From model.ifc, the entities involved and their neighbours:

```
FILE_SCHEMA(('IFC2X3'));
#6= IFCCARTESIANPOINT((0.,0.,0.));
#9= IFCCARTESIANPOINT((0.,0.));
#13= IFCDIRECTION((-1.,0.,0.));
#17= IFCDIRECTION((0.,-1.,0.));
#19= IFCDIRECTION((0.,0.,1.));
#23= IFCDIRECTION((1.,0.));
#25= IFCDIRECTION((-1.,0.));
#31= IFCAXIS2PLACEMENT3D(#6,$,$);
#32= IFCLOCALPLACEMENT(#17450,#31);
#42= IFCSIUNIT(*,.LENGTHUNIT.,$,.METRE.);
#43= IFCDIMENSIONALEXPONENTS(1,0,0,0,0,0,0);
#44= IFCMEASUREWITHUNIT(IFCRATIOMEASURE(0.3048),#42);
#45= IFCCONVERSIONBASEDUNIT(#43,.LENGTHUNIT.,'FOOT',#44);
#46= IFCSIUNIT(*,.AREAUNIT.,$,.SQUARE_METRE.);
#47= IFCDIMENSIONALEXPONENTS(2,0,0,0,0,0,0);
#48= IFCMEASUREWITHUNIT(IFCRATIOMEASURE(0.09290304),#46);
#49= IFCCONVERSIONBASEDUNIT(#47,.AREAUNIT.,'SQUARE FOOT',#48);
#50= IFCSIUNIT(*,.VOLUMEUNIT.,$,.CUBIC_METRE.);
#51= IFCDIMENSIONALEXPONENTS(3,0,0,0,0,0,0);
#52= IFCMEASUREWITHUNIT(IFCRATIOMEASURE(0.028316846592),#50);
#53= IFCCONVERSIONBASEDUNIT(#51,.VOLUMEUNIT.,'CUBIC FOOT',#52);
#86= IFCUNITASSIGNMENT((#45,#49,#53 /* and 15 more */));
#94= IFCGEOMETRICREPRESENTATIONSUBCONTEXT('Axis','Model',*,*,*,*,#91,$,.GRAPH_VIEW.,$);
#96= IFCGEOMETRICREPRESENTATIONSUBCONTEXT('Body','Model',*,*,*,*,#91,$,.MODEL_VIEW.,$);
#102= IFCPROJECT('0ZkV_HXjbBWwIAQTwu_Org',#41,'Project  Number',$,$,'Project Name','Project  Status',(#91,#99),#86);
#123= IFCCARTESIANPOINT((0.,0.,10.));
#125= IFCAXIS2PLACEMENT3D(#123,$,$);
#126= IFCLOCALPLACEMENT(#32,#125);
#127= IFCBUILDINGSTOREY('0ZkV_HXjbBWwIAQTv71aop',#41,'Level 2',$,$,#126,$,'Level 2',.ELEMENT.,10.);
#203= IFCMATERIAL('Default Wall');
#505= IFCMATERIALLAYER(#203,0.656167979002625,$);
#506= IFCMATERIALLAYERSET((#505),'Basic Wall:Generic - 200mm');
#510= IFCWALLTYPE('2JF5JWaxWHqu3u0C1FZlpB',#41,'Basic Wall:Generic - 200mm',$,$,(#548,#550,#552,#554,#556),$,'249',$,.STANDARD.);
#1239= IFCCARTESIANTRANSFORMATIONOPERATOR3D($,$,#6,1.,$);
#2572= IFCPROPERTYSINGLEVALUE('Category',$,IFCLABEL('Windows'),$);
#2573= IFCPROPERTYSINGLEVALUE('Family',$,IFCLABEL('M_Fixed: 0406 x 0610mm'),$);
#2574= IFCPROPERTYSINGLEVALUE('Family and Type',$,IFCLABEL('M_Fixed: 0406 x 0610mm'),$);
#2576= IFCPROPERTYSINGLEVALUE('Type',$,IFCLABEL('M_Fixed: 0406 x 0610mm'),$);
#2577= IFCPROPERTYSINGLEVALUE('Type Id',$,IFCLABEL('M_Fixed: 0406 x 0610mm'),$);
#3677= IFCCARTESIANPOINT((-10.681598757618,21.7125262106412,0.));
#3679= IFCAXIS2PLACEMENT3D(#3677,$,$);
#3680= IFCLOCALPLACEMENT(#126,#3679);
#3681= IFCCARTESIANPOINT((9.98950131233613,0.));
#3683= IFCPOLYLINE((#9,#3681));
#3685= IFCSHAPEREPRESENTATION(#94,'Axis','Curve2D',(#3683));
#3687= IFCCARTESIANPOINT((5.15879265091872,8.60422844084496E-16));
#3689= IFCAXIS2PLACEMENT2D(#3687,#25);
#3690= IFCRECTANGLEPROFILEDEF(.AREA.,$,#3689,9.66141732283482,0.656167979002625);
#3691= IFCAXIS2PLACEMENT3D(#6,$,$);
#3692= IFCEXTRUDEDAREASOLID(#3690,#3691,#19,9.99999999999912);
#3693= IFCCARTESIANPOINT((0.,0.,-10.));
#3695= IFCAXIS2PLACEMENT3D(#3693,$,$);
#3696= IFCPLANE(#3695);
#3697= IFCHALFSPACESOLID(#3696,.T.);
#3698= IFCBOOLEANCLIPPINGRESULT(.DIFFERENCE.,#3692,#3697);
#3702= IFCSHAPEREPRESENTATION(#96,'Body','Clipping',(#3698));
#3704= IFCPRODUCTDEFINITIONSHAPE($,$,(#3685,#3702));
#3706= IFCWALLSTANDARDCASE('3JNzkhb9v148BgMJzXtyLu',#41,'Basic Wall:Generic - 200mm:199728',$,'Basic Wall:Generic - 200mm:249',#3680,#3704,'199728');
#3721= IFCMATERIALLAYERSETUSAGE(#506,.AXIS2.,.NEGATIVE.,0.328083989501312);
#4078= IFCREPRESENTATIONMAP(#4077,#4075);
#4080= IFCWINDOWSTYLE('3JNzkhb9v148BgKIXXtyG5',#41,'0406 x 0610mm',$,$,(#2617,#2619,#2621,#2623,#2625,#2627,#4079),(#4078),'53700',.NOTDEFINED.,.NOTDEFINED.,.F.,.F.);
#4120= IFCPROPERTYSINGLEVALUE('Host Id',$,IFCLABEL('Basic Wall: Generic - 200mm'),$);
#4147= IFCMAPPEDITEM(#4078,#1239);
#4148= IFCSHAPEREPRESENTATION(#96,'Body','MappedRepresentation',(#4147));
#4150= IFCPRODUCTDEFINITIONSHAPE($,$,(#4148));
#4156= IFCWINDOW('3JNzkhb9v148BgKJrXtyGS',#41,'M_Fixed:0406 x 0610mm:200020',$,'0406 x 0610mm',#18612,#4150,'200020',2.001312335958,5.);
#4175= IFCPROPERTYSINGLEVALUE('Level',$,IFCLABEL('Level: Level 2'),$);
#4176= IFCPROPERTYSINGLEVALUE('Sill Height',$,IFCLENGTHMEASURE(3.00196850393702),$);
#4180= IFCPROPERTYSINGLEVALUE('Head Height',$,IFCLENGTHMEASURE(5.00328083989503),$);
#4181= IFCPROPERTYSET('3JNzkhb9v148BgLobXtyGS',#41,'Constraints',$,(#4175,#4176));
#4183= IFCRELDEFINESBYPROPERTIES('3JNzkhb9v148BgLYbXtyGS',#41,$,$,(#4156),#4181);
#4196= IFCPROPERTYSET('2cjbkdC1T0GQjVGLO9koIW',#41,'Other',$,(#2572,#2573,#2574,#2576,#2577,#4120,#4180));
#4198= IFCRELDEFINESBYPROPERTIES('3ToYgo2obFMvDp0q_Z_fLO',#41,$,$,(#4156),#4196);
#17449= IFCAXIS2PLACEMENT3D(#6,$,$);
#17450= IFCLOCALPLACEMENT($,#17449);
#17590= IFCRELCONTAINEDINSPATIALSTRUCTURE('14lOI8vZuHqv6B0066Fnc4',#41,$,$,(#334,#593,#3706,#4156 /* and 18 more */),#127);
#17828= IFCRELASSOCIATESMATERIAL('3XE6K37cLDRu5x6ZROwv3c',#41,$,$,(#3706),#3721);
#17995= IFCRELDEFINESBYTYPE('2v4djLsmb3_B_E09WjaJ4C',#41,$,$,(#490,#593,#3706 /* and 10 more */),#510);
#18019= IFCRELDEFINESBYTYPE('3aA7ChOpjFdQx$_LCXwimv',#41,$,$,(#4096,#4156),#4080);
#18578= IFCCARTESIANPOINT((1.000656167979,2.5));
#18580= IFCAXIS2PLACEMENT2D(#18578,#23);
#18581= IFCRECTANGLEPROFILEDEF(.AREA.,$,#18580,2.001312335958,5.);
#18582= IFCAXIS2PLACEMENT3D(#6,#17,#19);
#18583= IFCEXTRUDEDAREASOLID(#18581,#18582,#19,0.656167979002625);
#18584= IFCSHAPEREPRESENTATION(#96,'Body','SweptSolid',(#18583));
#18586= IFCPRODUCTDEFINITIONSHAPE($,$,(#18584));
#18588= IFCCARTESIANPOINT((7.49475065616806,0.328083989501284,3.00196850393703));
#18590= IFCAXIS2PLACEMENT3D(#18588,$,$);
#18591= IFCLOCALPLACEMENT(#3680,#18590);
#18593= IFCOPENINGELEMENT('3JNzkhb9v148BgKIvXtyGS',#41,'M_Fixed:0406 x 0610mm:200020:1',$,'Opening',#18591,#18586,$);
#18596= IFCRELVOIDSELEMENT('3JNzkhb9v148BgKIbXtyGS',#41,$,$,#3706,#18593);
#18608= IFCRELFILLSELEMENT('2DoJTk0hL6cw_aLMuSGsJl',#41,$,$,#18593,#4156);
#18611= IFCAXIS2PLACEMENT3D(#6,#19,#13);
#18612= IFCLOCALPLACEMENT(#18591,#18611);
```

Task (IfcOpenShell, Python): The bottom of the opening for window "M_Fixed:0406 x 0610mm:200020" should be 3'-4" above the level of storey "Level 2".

```python
import numpy as np
import ifcopenshell
import ifcopenshell.api.geometry
import ifcopenshell.api.pset
import ifcopenshell.geom
import ifcopenshell.util.element
import ifcopenshell.util.placement
import ifcopenshell.util.shape
import ifcopenshell.util.unit

model = ifcopenshell.open("model.ifc")
unit_scale = ifcopenshell.util.unit.calculate_unit_scale(model)

window = model.by_guid("3JNzkhb9v148BgKJrXtyGS")
opening = window.FillsVoids[0].RelatingOpeningElement
storey = ifcopenshell.util.element.get_container(window, ifc_class="IfcBuildingStorey")
level = ifcopenshell.util.placement.get_local_placement(storey.ObjectPlacement)[2, 3]

# The opening's origin need not be at the sill, so measure its lowest point.
shape = ifcopenshell.geom.create_shape(ifcopenshell.geom.settings(), opening)
bottom = ifcopenshell.util.shape.get_shape_bottom_elevation(shape, shape.geometry) / unit_scale
dz = level + 40 * 0.0254 / unit_scale - bottom

shift = np.array([0.0, 0.0, dz])
# The window is placed relative to its opening, so it follows when the opening moves.
matrix = ifcopenshell.util.placement.get_local_placement(opening.ObjectPlacement)
matrix[:3, 3] += shift
ifcopenshell.api.geometry.edit_object_placement(
    model, product=opening, matrix=matrix, is_si=False, should_transform_children=True
)

# Keep the stored heights in step.
pset = model.by_id(ifcopenshell.util.element.get_pset(window, "Constraints", should_inherit=False)["id"])
ifcopenshell.api.pset.edit_pset(model, pset=pset, properties={
    "Sill Height": model.create_entity("IfcLengthMeasure", ifcopenshell.util.element.get_pset(window, "Constraints", "Sill Height") + dz),
})
pset = model.by_id(ifcopenshell.util.element.get_pset(window, "Other", should_inherit=False)["id"])
ifcopenshell.api.pset.edit_pset(model, pset=pset, properties={
    "Head Height": model.create_entity("IfcLengthMeasure", ifcopenshell.util.element.get_pset(window, "Other", "Head Height") + dz),
})

print(f"moved by {dz * unit_scale:+.3f} m")

model.write("model_updated.ifc")
```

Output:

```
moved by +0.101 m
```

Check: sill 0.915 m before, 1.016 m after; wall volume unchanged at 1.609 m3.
